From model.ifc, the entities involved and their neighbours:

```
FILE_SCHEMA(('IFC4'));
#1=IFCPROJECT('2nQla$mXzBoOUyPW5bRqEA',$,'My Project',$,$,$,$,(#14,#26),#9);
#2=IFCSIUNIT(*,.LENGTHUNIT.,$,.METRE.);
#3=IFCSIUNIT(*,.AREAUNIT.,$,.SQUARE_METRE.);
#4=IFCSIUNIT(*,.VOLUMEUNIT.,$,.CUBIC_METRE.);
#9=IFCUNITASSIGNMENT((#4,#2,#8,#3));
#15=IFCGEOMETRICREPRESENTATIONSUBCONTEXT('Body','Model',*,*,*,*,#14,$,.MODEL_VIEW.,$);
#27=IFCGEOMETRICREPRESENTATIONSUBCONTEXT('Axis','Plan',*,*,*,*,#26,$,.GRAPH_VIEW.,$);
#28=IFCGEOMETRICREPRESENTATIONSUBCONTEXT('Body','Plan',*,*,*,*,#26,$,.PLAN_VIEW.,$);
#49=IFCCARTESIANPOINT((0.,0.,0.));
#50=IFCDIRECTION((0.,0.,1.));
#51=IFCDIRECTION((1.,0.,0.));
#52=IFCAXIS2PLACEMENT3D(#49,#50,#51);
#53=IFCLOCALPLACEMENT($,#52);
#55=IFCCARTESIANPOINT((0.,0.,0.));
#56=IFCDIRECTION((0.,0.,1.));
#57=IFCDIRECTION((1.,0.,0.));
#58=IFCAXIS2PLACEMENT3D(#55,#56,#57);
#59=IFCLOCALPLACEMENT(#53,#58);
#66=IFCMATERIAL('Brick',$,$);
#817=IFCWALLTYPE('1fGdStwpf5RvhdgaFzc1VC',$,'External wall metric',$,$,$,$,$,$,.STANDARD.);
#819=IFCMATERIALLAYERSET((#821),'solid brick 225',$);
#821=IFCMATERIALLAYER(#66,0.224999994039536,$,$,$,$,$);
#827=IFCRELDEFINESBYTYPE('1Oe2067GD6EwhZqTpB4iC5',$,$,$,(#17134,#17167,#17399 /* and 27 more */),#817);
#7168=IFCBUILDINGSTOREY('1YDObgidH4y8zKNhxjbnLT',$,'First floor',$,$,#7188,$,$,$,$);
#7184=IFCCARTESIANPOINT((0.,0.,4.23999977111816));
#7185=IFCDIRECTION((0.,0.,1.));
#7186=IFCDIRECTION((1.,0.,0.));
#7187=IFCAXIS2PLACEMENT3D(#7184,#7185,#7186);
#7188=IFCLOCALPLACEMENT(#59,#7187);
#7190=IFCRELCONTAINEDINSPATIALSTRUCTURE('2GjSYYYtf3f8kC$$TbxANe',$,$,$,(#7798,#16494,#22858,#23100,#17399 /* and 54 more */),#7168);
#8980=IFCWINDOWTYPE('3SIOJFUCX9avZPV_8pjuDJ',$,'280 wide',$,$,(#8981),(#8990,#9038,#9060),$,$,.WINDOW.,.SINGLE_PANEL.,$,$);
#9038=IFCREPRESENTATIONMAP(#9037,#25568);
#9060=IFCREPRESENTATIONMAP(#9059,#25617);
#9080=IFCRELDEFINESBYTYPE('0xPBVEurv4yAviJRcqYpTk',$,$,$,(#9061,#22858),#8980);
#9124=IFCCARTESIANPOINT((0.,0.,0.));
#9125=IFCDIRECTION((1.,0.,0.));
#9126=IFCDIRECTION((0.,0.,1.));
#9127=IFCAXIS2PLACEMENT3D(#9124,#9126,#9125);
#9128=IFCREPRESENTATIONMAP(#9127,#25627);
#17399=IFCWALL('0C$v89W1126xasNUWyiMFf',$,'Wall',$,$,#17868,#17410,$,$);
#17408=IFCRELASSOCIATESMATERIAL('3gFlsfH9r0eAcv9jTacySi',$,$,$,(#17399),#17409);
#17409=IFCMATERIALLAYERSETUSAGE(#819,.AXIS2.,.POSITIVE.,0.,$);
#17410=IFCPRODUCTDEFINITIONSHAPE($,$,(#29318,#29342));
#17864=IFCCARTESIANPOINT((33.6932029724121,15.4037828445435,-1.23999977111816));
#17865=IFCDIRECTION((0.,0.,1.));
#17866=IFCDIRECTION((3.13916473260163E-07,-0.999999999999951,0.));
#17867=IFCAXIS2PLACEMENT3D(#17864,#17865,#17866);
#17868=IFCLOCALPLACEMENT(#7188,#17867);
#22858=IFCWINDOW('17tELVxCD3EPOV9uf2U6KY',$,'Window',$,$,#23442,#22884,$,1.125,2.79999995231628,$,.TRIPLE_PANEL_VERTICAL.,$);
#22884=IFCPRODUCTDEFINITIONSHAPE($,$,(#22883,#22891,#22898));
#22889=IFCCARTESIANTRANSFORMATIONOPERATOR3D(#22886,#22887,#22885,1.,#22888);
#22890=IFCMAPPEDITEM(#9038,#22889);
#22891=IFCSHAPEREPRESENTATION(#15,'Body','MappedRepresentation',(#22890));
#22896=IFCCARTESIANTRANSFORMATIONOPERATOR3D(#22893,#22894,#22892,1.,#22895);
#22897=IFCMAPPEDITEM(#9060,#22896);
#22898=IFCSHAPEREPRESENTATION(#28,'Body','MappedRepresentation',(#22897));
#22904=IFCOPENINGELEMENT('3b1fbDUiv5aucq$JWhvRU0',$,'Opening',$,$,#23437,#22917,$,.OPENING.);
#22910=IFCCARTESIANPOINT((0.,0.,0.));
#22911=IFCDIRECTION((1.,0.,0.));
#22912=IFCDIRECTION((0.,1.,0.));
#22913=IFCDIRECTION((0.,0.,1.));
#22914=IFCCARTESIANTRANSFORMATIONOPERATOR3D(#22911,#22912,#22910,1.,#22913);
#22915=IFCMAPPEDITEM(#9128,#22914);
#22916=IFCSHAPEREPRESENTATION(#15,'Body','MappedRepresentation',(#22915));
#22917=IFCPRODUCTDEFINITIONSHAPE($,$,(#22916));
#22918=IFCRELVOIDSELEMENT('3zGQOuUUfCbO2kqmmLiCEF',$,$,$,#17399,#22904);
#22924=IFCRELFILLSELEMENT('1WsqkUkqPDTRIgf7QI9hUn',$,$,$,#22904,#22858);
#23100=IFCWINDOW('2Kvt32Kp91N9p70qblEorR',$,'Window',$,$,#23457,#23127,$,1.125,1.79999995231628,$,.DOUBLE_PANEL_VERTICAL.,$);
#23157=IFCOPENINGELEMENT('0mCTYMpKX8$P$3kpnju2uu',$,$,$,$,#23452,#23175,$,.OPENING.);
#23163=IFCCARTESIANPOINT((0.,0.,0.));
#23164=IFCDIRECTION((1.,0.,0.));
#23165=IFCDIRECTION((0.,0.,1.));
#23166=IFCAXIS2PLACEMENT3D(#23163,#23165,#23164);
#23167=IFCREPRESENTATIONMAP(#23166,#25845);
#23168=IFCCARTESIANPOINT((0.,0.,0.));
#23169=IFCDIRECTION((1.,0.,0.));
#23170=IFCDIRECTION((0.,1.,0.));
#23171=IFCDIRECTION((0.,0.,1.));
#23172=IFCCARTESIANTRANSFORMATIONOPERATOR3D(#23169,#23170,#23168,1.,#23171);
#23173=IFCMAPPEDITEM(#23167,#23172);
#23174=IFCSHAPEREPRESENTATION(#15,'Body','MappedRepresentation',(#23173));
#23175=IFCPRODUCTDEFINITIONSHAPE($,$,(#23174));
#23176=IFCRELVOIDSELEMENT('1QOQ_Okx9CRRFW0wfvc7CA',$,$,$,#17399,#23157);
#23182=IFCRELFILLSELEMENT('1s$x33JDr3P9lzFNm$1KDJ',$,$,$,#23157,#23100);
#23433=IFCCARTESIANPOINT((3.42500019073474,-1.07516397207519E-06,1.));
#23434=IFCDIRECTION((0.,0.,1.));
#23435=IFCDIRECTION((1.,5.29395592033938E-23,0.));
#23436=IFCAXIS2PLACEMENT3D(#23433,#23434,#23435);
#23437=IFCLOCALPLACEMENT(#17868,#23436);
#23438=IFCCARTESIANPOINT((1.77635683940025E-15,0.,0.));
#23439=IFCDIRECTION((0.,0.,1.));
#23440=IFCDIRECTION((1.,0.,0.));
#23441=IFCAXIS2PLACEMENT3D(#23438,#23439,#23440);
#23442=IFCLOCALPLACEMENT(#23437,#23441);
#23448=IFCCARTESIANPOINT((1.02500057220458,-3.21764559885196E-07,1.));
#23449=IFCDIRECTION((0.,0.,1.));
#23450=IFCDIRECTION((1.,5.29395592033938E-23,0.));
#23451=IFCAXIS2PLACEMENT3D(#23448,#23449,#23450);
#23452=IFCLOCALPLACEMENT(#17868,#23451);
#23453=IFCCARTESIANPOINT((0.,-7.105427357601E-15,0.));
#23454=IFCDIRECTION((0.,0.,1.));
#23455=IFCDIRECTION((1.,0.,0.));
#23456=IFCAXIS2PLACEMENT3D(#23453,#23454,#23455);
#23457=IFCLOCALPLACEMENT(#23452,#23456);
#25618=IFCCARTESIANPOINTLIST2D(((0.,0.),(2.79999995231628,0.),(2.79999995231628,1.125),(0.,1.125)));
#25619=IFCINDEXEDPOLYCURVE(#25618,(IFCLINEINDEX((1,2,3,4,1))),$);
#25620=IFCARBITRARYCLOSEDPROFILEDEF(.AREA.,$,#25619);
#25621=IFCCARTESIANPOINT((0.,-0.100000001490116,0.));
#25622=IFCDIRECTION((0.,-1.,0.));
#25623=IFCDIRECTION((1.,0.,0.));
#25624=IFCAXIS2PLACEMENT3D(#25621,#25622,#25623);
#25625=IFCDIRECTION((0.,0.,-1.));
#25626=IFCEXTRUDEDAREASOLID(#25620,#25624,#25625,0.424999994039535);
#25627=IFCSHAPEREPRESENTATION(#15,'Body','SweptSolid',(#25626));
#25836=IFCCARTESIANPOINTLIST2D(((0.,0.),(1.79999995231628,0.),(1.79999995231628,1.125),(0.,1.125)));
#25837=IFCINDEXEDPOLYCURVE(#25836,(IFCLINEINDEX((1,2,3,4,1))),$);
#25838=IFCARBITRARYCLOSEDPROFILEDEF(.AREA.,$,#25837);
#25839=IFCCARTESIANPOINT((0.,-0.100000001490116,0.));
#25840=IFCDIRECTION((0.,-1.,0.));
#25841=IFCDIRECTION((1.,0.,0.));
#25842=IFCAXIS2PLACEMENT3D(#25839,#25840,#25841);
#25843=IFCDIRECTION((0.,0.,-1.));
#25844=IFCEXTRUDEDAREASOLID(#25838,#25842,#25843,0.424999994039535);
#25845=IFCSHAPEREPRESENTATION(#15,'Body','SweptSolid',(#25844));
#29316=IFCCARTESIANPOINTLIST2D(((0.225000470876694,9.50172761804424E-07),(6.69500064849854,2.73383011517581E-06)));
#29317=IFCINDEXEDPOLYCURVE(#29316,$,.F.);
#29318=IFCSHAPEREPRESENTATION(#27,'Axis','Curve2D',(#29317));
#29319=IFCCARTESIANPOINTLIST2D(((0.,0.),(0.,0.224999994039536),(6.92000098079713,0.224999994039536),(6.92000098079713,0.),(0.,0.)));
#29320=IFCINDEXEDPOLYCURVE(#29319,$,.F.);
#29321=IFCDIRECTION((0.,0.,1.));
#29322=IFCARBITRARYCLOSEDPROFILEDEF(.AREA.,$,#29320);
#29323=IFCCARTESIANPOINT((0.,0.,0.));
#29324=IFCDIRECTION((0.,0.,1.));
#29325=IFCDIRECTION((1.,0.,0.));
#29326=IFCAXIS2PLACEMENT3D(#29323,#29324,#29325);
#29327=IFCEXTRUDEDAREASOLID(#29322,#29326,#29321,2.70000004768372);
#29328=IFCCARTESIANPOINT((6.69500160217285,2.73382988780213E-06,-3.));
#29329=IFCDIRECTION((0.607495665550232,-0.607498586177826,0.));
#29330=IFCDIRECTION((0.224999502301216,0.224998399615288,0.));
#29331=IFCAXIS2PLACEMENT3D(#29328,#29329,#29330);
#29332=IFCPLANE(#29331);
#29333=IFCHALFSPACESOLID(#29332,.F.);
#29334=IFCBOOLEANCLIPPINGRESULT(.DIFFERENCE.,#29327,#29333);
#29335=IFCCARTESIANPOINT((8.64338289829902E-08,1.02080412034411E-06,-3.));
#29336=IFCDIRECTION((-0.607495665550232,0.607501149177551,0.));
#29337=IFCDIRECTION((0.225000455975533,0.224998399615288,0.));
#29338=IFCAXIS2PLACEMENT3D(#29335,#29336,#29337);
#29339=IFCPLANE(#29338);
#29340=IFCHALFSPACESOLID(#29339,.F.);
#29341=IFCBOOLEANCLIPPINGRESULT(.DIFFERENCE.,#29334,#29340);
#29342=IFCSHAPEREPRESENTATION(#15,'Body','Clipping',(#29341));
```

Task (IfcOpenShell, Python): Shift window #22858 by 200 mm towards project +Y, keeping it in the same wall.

```python
import ifcopenshell
import ifcopenshell.api.geometry
import ifcopenshell.util.placement

model = ifcopenshell.open("model.ifc")

window = model.by_id(22858)
opening = window.FillsVoids[0].RelatingOpeningElement
wall = opening.VoidsElements[0].RelatingBuildingElement

wall_matrix = ifcopenshell.util.placement.get_local_placement(wall.ObjectPlacement)
shift = wall_matrix[:3, 0] * -0.2
before = ifcopenshell.util.placement.get_local_placement(window.ObjectPlacement)[:3, 3].copy()

# The window is placed relative to its opening, so it follows when the opening moves.
matrix = ifcopenshell.util.placement.get_local_placement(opening.ObjectPlacement)
matrix[:3, 3] += shift
ifcopenshell.api.geometry.edit_object_placement(
    model, product=opening, matrix=matrix, is_si=False, should_transform_children=True
)

after = ifcopenshell.util.placement.get_local_placement(window.ObjectPlacement)[:3, 3]
print("window moved by", (after - before).round(3) + 0.0)

model.write("model_updated.ifc")
```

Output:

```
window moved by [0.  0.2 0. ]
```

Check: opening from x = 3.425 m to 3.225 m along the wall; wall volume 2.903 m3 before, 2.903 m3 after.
